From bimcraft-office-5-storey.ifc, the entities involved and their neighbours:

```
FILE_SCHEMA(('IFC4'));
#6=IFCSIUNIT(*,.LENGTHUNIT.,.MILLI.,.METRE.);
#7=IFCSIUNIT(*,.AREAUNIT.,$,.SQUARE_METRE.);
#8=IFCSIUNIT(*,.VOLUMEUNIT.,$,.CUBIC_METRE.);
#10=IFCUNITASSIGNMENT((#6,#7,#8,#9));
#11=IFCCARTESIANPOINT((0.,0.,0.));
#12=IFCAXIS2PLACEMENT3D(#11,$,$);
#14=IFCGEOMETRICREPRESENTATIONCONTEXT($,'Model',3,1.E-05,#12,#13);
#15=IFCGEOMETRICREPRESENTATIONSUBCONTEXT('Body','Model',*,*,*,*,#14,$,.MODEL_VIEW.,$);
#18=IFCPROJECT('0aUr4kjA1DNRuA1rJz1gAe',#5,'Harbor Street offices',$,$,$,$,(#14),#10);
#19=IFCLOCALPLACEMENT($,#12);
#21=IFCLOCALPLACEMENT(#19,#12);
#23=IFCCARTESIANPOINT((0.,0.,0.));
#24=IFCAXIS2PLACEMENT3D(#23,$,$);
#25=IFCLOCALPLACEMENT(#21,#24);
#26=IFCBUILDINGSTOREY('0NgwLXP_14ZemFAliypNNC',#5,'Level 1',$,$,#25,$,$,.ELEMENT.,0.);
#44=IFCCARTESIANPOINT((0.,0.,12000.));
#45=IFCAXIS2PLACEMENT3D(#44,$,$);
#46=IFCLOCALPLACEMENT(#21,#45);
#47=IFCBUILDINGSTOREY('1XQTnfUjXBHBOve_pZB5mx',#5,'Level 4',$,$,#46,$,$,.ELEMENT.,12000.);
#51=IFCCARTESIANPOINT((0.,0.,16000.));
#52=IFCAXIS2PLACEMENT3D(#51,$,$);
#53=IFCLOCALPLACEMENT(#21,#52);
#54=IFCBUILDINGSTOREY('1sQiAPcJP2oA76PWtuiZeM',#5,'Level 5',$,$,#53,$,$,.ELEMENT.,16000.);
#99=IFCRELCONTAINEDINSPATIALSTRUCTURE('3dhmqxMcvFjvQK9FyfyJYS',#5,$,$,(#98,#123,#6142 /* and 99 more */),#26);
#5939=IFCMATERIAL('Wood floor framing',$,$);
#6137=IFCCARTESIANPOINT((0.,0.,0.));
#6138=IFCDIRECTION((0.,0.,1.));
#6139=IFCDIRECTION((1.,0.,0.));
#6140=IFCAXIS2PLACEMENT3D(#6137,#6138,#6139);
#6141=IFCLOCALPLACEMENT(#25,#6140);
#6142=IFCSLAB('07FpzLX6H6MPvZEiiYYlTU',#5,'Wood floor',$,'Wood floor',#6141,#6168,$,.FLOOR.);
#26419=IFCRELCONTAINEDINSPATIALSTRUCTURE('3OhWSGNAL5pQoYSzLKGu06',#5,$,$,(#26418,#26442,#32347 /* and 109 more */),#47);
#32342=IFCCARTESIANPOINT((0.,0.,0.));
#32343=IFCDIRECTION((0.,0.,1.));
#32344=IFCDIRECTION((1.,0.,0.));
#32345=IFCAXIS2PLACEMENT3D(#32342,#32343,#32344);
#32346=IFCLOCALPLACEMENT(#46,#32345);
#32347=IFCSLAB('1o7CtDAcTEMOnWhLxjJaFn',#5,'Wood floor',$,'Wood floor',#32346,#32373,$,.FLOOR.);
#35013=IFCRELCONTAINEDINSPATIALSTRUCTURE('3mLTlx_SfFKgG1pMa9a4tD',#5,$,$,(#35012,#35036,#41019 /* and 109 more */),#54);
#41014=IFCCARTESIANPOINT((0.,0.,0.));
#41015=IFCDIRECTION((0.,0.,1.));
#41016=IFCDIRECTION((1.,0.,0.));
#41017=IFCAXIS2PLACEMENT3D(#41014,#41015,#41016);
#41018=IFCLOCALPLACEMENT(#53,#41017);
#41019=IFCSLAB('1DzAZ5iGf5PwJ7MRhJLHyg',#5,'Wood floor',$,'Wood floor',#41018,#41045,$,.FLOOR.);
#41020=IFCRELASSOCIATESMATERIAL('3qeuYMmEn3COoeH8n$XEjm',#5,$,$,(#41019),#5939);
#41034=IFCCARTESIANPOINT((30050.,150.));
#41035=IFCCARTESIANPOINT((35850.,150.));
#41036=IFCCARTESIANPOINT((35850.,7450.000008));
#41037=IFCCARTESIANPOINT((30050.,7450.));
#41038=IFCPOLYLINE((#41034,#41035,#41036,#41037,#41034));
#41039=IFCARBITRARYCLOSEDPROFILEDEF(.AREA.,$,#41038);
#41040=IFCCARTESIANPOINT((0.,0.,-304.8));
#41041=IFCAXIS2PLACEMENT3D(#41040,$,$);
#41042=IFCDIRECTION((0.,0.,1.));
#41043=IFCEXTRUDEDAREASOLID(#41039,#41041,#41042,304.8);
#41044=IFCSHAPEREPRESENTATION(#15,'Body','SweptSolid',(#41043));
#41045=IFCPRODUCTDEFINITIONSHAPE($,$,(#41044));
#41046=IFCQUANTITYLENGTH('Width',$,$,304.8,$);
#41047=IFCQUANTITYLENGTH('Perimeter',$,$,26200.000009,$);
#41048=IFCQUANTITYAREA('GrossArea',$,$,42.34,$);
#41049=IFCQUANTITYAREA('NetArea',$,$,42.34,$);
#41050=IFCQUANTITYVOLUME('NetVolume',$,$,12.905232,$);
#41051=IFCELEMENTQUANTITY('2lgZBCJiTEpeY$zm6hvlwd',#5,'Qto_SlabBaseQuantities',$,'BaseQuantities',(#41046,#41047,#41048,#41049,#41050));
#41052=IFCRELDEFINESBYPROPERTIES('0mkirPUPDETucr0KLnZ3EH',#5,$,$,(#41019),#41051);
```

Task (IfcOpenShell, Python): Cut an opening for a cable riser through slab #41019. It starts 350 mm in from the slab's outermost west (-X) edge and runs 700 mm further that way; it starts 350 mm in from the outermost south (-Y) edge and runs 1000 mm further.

```python
import numpy as np
import ifcopenshell
import ifcopenshell.api.feature
import ifcopenshell.api.geometry
import ifcopenshell.api.pset
import ifcopenshell.api.root
import ifcopenshell.geom
import ifcopenshell.util.element
import ifcopenshell.util.placement
import ifcopenshell.util.representation
import ifcopenshell.util.shape
import ifcopenshell.util.unit

model = ifcopenshell.open("bimcraft-office-5-storey.ifc")
unit_scale = ifcopenshell.util.unit.calculate_unit_scale(model)
area_scale = ifcopenshell.util.unit.calculate_unit_scale(model, "AREAUNIT")
volume_scale = ifcopenshell.util.unit.calculate_unit_scale(model, "VOLUMEUNIT")
settings = ifcopenshell.geom.settings()


def volume(element):
    """Net volume in cubic metres, openings subtracted."""
    shape = ifcopenshell.geom.create_shape(settings, element)
    return ifcopenshell.util.shape.get_volume(shape.geometry)


slab = model.by_guid("1DzAZ5iGf5PwJ7MRhJLHyg")
before = volume(slab)

# Extent in the slab's own axes, in metres. The edges named are its -X and -Y sides.
slab_shape = ifcopenshell.geom.create_shape(settings, slab)
vertices = ifcopenshell.util.shape.get_vertices(slab_shape.geometry)
x_min, y_min, bottom = vertices.min(axis=0)
top = vertices[:, 2].max()

opening = ifcopenshell.api.root.create_entity(model, ifc_class="IfcOpeningElement", name="Cable riser opening", predefined_type="OPENING")
context = ifcopenshell.util.representation.get_context(model, "Model", "Body", "MODEL_VIEW")
width, depth = 0.7, 1
outline = [(0.0, 0.0), (width, 0.0), (width, depth), (0.0, depth), (0.0, 0.0)]
# Overshoot both faces by 50 mm so the cut is clean.
shape = ifcopenshell.api.geometry.add_slab_representation(
    model, context=context, depth=top - bottom + 0.1, polyline=outline
)
ifcopenshell.api.geometry.assign_representation(model, product=opening, representation=shape)

matrix = ifcopenshell.util.placement.get_local_placement(slab.ObjectPlacement)
matrix[:, 3] = matrix @ np.append(np.array([x_min + 0.35, y_min + 0.35, bottom - 0.05]) / unit_scale, 1.0)
ifcopenshell.api.geometry.edit_object_placement(model, product=opening, matrix=matrix, is_si=False)
ifcopenshell.api.feature.add_feature(model, feature=opening, element=slab)

after = volume(slab)

# Update the slab's stored quantities.
qto = model.by_id(ifcopenshell.util.element.get_pset(slab, "Qto_SlabBaseQuantities", should_inherit=False)["id"])
ifcopenshell.api.pset.edit_qto(model, qto=qto, properties={
    "NetArea": after / (top - bottom) / area_scale,
    "NetVolume": after / volume_scale,
})

print(f"slab volume {before:.3f} -> {after:.3f} m3")

model.write("bimcraft-office-5-storey_updated.ifc")
```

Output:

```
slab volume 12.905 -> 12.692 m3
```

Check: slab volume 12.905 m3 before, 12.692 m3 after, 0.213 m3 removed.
